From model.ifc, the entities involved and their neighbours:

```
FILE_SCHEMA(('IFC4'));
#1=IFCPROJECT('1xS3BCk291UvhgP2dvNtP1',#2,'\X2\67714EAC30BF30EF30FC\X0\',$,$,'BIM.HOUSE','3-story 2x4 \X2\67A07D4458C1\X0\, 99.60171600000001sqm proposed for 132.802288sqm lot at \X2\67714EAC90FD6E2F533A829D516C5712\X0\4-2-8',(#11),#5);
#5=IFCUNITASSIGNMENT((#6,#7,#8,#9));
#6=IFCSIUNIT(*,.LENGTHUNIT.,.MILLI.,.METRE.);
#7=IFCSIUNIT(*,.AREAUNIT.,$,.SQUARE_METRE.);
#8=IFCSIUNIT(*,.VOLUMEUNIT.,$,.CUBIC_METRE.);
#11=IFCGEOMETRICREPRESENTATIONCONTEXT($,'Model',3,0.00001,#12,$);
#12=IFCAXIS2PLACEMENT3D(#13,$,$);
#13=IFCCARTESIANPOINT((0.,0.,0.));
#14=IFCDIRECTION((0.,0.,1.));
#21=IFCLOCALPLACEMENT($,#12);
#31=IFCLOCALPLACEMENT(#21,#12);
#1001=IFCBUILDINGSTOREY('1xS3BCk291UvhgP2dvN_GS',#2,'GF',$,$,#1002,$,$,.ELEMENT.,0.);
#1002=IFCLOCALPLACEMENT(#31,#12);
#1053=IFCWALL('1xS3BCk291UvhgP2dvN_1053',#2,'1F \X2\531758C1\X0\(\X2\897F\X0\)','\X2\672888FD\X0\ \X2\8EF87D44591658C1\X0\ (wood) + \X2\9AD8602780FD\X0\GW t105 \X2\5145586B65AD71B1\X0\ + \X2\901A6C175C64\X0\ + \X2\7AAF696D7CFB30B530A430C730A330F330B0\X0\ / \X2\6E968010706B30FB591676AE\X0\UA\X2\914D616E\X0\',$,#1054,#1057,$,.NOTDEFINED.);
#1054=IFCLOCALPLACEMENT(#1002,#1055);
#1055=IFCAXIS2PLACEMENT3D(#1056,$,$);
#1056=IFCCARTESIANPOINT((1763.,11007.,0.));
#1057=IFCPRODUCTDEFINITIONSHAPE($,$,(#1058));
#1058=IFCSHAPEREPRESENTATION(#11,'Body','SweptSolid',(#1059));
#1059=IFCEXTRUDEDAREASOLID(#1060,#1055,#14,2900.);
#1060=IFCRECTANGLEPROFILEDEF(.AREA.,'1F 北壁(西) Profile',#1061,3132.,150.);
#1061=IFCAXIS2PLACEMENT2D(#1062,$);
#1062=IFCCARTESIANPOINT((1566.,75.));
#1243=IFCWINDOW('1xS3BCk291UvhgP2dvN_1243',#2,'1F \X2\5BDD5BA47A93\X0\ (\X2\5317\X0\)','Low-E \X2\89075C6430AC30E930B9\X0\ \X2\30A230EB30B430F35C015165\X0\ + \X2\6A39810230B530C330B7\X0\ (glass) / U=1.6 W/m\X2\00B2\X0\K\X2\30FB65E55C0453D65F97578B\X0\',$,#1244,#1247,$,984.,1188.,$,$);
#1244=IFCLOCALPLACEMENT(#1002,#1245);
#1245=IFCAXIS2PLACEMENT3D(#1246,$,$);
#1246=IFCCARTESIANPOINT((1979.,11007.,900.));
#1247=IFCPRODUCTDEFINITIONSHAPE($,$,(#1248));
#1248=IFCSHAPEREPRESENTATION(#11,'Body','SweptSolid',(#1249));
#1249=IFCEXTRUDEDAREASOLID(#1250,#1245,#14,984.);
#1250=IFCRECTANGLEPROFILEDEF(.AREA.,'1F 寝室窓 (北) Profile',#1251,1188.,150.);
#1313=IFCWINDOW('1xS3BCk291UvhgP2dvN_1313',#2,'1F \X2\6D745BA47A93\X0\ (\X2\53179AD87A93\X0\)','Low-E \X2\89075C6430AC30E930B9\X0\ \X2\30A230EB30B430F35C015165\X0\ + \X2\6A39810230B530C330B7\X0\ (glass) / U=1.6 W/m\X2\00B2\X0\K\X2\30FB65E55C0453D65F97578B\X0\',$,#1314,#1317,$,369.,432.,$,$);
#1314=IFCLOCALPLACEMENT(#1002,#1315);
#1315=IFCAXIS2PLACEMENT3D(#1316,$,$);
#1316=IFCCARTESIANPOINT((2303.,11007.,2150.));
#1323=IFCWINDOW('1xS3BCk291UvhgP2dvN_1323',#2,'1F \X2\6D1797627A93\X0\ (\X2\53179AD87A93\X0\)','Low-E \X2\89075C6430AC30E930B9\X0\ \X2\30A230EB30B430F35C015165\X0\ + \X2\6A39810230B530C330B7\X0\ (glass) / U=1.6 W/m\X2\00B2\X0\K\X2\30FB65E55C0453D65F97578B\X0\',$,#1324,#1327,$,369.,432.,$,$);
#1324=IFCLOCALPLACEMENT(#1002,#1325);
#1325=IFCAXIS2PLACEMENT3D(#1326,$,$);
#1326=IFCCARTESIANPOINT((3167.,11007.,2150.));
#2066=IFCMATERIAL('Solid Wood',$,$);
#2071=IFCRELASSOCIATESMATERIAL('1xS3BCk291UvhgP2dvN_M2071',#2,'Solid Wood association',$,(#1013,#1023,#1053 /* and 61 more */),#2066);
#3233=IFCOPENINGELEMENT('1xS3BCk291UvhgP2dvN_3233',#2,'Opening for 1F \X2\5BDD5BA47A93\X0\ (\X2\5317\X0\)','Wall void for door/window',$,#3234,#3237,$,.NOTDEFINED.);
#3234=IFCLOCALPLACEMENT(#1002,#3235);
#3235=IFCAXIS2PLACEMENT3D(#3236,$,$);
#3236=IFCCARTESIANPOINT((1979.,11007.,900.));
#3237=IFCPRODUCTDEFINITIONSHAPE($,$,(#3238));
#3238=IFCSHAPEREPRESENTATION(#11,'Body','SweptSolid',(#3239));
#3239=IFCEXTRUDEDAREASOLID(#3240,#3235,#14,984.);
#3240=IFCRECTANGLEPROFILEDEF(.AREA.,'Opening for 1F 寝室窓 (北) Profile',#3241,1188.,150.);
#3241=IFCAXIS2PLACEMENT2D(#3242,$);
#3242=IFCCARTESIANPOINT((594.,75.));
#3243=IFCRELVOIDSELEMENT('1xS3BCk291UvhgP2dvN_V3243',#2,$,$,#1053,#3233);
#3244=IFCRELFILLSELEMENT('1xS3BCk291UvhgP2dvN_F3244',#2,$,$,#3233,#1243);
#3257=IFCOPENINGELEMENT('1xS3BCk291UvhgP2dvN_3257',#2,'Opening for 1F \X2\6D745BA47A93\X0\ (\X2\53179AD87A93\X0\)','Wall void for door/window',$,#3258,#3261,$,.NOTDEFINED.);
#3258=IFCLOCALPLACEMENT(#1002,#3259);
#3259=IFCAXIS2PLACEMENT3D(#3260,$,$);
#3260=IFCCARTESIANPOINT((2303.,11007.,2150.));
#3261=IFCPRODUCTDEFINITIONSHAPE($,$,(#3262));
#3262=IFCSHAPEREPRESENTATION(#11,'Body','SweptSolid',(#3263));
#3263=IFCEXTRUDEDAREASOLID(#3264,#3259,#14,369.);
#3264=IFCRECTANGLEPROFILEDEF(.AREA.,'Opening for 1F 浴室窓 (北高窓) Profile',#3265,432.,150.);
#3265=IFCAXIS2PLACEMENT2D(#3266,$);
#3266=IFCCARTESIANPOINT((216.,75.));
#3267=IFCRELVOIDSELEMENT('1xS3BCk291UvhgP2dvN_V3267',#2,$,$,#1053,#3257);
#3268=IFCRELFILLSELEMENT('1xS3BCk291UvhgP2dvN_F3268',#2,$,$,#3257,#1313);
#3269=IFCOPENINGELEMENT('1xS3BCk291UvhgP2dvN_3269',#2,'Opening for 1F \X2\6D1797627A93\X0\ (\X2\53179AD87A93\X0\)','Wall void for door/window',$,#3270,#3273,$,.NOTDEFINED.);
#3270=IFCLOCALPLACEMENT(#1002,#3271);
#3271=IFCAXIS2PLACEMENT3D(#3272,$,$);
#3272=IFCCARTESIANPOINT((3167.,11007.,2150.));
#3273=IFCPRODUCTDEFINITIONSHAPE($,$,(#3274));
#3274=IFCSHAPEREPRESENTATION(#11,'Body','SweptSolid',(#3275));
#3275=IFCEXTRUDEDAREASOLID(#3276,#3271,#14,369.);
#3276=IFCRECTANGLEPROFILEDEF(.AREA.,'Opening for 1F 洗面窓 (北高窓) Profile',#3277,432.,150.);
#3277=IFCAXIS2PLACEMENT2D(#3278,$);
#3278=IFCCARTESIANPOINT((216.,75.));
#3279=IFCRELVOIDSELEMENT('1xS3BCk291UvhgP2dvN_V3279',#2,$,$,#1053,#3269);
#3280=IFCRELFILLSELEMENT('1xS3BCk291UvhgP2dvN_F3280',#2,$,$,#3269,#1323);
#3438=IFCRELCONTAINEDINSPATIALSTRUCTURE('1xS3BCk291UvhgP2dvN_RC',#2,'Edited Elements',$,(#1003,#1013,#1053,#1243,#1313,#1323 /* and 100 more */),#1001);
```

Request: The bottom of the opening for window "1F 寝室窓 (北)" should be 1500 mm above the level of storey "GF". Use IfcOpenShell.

```python
import numpy as np
import ifcopenshell
import ifcopenshell.api.geometry
import ifcopenshell.geom
import ifcopenshell.util.element
import ifcopenshell.util.placement
import ifcopenshell.util.shape
import ifcopenshell.util.unit

model = ifcopenshell.open("model.ifc")
unit_scale = ifcopenshell.util.unit.calculate_unit_scale(model)

window = model.by_guid("1xS3BCk291UvhgP2dvN_1243")
opening = window.FillsVoids[0].RelatingOpeningElement
storey = ifcopenshell.util.element.get_container(window, ifc_class="IfcBuildingStorey")
level = ifcopenshell.util.placement.get_local_placement(storey.ObjectPlacement)[2, 3]

# The opening's origin need not be at the sill, so measure its lowest point.
shape = ifcopenshell.geom.create_shape(ifcopenshell.geom.settings(), opening)
bottom = ifcopenshell.util.shape.get_shape_bottom_elevation(shape, shape.geometry) / unit_scale
dz = level + 1500.0 - bottom

shift = np.array([0.0, 0.0, dz])
# The window is not placed relative to its opening, so move both.
for product in (opening, window):
    matrix = ifcopenshell.util.placement.get_local_placement(product.ObjectPlacement)
    matrix[:3, 3] += shift
    ifcopenshell.api.geometry.edit_object_placement(model, product=product, matrix=matrix, is_si=False)

print(f"moved by {dz * unit_scale:+.3f} m")

model.write("model_updated.ifc")
```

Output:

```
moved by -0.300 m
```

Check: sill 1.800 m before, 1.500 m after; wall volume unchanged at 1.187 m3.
